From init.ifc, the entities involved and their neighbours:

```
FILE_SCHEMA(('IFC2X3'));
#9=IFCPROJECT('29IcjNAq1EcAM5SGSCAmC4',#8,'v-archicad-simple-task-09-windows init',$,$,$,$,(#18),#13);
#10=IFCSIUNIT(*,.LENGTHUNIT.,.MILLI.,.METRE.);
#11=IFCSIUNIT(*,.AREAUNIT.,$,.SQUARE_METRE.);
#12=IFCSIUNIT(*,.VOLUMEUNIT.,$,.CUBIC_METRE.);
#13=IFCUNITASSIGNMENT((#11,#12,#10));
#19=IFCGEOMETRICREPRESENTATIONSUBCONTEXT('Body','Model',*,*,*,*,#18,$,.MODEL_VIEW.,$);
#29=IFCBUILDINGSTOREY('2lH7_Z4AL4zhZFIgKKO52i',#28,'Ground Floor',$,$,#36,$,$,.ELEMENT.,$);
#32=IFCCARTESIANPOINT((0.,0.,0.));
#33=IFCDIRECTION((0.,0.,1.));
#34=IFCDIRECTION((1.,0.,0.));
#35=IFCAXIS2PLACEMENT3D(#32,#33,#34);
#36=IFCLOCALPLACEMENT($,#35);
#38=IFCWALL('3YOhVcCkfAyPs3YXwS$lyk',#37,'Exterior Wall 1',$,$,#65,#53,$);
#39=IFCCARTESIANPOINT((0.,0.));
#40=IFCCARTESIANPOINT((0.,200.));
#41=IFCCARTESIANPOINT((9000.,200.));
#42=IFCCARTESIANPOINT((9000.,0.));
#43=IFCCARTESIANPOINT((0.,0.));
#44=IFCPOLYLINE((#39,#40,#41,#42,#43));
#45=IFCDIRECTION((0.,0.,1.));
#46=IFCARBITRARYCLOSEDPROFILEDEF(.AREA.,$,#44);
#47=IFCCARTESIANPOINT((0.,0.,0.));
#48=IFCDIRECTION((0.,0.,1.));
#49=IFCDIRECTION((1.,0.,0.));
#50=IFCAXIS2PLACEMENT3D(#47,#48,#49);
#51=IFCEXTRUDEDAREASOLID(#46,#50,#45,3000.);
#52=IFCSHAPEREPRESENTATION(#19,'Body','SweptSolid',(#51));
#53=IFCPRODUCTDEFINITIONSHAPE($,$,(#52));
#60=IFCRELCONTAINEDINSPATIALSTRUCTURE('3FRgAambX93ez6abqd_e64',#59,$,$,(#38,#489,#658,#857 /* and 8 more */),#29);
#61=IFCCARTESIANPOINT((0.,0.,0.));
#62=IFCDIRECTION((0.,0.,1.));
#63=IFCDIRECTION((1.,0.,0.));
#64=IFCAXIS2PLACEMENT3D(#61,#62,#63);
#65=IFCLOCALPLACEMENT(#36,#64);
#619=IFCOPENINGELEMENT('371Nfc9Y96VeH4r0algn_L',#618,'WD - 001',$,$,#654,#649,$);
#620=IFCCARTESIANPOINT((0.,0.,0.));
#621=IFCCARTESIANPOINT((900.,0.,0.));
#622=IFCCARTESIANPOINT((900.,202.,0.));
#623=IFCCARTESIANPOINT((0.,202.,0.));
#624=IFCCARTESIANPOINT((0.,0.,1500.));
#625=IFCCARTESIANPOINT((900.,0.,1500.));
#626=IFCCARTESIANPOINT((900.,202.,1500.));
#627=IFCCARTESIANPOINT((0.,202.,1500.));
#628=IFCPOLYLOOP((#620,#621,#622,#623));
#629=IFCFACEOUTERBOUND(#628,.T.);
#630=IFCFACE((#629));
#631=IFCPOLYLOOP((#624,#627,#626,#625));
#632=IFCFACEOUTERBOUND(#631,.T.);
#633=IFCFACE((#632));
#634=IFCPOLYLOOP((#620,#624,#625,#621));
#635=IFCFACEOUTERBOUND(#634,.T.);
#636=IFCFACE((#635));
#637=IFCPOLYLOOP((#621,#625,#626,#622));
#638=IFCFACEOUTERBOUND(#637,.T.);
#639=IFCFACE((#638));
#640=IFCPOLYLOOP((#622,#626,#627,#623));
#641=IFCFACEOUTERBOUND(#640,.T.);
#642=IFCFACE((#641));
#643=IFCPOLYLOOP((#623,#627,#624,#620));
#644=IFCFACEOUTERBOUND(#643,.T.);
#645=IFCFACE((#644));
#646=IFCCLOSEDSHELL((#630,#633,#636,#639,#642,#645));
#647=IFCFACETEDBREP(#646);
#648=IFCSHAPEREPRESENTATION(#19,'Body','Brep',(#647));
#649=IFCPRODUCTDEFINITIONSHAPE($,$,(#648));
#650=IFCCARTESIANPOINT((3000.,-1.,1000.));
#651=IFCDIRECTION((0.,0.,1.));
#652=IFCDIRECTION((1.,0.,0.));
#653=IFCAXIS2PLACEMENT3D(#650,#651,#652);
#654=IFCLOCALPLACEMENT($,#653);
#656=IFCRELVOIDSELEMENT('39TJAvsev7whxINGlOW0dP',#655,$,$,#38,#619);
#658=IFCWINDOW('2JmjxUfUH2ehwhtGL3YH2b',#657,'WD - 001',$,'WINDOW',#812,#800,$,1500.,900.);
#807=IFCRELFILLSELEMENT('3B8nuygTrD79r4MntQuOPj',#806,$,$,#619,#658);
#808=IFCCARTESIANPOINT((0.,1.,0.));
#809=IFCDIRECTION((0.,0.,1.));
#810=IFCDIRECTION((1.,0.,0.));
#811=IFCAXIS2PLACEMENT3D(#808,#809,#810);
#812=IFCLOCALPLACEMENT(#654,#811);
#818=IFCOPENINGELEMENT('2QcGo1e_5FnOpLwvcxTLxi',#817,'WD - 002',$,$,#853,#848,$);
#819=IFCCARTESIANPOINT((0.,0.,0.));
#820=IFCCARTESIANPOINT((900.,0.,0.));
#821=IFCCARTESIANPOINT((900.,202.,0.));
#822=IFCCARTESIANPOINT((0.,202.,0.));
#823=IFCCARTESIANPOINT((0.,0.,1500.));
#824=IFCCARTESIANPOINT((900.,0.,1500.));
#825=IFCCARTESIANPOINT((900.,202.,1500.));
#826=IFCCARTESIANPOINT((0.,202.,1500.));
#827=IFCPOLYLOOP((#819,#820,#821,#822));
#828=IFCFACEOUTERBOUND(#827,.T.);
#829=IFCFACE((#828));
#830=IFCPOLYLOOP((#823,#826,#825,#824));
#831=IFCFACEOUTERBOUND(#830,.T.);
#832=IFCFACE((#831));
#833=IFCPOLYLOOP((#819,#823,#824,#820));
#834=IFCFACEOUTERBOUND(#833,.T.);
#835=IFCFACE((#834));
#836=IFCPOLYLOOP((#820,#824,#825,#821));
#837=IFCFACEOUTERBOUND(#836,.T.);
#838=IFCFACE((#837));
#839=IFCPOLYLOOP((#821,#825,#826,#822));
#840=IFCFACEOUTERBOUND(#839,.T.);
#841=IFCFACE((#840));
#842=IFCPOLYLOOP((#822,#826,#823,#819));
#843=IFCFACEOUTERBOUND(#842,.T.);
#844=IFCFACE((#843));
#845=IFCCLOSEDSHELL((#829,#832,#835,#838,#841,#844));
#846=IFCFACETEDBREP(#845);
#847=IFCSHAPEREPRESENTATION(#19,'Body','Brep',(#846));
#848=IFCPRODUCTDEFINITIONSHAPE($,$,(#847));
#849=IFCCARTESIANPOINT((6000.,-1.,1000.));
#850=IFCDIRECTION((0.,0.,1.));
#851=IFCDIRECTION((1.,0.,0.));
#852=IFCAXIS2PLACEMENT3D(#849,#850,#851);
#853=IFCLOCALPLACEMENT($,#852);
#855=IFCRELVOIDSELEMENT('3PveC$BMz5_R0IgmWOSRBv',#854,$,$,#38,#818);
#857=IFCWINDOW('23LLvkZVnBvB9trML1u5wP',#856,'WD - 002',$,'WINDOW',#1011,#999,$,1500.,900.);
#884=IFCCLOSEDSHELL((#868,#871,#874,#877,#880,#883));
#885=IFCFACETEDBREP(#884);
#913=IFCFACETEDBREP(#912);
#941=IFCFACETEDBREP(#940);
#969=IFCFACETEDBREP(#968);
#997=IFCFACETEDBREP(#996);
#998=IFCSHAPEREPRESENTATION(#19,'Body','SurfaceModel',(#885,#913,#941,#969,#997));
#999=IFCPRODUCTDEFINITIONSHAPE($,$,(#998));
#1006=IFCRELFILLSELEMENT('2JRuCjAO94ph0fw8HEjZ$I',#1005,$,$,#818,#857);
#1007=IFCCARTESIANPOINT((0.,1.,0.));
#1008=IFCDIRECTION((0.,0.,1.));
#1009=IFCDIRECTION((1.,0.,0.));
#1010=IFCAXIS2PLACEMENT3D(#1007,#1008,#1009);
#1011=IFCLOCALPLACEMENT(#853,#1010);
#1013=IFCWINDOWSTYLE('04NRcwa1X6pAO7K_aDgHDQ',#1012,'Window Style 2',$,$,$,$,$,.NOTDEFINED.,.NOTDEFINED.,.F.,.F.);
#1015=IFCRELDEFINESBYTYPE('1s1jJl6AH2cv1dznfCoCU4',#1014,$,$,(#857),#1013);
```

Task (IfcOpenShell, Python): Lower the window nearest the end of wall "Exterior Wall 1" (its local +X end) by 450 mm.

```python
import numpy as np
import ifcopenshell
import ifcopenshell.api.geometry
import ifcopenshell.util.placement
import ifcopenshell.util.unit

model = ifcopenshell.open("init.ifc")
unit_scale = ifcopenshell.util.unit.calculate_unit_scale(model)

window = model.by_guid("23LLvkZVnBvB9trML1u5wP")
opening = window.FillsVoids[0].RelatingOpeningElement
dz = -0.45 / unit_scale

shift = np.array([0.0, 0.0, dz])
# The window is placed relative to its opening, so it follows when the opening moves.
matrix = ifcopenshell.util.placement.get_local_placement(opening.ObjectPlacement)
matrix[:3, 3] += shift
ifcopenshell.api.geometry.edit_object_placement(
    model, product=opening, matrix=matrix, is_si=False, should_transform_children=True
)

print(f"moved by {dz * unit_scale:+.3f} m")

model.write("init_edited.ifc")
```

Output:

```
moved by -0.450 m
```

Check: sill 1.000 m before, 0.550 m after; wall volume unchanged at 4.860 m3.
